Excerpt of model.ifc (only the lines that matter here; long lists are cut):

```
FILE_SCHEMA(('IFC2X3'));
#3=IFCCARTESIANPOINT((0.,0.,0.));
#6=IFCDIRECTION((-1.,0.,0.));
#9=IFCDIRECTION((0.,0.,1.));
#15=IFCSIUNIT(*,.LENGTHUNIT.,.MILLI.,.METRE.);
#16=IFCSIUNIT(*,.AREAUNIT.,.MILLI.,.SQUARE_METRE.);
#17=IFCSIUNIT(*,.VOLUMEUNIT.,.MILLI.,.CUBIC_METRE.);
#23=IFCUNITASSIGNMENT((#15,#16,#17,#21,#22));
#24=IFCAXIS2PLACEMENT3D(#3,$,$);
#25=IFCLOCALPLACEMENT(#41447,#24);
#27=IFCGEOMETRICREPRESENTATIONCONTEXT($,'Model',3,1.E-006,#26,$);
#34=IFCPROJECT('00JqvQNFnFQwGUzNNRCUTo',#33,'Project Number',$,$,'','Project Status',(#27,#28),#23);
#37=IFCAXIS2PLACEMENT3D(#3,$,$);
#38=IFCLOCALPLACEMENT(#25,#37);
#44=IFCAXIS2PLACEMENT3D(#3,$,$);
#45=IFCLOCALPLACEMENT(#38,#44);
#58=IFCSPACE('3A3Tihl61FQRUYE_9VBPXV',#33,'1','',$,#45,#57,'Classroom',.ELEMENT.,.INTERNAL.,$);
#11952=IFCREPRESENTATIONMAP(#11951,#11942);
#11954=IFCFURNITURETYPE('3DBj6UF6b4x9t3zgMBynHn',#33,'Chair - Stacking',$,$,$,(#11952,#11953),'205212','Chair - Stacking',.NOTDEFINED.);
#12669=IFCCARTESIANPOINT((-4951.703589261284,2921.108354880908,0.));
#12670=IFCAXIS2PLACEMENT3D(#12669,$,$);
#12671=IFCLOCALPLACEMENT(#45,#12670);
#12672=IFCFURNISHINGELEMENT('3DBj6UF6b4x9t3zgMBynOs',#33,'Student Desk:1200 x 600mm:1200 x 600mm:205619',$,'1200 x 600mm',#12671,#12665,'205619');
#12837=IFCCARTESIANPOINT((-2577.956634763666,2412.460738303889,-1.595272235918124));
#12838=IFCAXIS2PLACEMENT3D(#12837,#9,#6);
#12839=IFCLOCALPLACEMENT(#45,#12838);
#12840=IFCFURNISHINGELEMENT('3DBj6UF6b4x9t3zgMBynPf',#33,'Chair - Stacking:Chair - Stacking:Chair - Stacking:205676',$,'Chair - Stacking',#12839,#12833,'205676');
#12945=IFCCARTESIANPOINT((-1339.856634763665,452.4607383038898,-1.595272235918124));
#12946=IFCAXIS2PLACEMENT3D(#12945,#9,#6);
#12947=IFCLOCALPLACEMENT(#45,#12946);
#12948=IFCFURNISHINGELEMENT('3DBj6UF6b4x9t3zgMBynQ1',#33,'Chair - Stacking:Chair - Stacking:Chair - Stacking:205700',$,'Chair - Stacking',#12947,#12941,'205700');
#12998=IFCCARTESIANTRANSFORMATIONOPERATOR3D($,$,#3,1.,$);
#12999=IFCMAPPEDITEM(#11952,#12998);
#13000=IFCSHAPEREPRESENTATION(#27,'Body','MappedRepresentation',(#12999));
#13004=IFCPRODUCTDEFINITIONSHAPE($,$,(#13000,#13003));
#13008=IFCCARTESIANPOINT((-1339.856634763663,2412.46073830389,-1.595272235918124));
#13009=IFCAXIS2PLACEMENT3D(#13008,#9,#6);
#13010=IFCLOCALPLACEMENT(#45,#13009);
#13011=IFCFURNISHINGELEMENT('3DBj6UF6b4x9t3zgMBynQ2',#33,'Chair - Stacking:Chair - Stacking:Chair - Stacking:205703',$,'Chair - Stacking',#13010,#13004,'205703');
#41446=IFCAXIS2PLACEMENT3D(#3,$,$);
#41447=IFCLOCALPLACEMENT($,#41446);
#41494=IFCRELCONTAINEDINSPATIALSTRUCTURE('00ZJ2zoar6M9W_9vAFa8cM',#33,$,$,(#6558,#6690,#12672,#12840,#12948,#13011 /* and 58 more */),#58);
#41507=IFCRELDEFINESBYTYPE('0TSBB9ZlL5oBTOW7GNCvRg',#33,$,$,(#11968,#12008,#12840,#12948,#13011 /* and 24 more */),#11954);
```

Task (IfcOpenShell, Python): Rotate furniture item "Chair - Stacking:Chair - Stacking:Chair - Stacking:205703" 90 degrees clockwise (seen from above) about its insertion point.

```python
import ifcopenshell
import ifcopenshell.api.geometry
import ifcopenshell.util.placement

model = ifcopenshell.open("model.ifc")

item = model.by_id(13011)
matrix = ifcopenshell.util.placement.get_local_placement(item.ObjectPlacement)
matrix = matrix @ ifcopenshell.util.placement.rotation(-90, "Z")
ifcopenshell.api.geometry.edit_object_placement(model, product=item, matrix=matrix, is_si=False)

print(ifcopenshell.util.placement.get_local_placement(item.ObjectPlacement).round(3) + 0.0)

model.write("model_updated.ifc")
```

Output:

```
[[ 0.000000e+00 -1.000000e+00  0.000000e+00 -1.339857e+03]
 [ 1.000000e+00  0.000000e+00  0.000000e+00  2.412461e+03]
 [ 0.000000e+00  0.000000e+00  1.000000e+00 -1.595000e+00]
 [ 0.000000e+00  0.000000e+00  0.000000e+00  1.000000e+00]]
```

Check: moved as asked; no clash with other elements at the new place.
